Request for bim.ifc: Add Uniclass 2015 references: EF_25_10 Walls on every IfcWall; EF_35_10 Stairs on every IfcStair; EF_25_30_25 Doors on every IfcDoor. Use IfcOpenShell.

First a look at what the model holds.

```python
import ifcopenshell

model = ifcopenshell.open("bim.ifc")
print(model.schema)
print("classifications:", [c.Name for c in model.by_type("IfcClassification")])
for ifc_class in ("IfcDoor", "IfcRoof", "IfcStair", "IfcWall", "IfcWindow"):
    print(ifc_class, len(model.by_type(ifc_class)))
```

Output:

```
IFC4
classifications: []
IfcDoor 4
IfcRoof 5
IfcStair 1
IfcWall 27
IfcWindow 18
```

```python
import ifcopenshell
import ifcopenshell.api.classification

model = ifcopenshell.open("bim.ifc")

system = ifcopenshell.api.classification.add_classification(model, classification="Uniclass 2015")

codes = {
    "IfcWall": ("EF_25_10", "Walls"),
    "IfcStair": ("EF_35_10", "Stairs"),
    "IfcDoor": ("EF_25_30_25", "Doors"),
}
for ifc_class, (code, name) in codes.items():
    products = model.by_type(ifc_class)
    ifcopenshell.api.classification.add_reference(
        model, products=products, classification=system, identification=code, name=name
    )
    print(code, len(products))

model.write("bim-out.ifc")
```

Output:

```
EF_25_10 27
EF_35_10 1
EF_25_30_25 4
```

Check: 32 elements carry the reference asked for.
